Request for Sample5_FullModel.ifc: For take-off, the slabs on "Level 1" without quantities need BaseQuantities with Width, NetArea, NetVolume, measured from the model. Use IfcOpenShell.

First a look at what the model holds.

```python
import ifcopenshell
import ifcopenshell.util.element
import ifcopenshell.util.unit

model = ifcopenshell.open("Sample5_FullModel.ifc")
print(model.schema)
for unit_type in ("LENGTHUNIT", "AREAUNIT", "VOLUMEUNIT"):
    print(unit_type, ifcopenshell.util.unit.calculate_unit_scale(model, unit_type))
storey = next(s for s in model.by_type("IfcBuildingStorey") if s.Name == "Level 1")
slabs = [e for e in ifcopenshell.util.element.get_decomposition(storey) if e.is_a("IfcSlab")]
for e in sorted(slabs, key=lambda e: e.id()):
    print(e.id(), e.is_a(), e.Name, list(ifcopenshell.util.element.get_psets(e, qtos_only=True)), sep=" | ")
```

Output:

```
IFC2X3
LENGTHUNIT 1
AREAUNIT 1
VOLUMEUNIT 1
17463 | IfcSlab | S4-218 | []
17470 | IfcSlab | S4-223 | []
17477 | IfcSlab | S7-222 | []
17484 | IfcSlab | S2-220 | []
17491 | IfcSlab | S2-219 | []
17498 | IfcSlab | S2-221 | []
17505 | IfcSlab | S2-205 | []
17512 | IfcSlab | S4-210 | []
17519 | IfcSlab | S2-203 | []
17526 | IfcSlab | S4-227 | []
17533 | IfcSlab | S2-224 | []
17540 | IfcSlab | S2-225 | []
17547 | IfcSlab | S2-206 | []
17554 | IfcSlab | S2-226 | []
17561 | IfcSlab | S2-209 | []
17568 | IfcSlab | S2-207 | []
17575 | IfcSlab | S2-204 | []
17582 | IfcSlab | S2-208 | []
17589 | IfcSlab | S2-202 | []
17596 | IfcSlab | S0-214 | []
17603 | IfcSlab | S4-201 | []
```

```python
import ifcopenshell
import ifcopenshell.api.pset
import ifcopenshell.geom
import ifcopenshell.util.element
import ifcopenshell.util.shape
import ifcopenshell.util.unit

model = ifcopenshell.open("Sample5_FullModel.ifc")
unit_scale = ifcopenshell.util.unit.calculate_unit_scale(model)
area_scale = ifcopenshell.util.unit.calculate_unit_scale(model, "AREAUNIT")
volume_scale = ifcopenshell.util.unit.calculate_unit_scale(model, "VOLUMEUNIT")
settings = ifcopenshell.geom.settings()

storey = next(s for s in model.by_type("IfcBuildingStorey") if s.Name == "Level 1")
slabs = [e for e in ifcopenshell.util.element.get_decomposition(storey) if e.is_a("IfcSlab")]

for e in sorted(slabs, key=lambda e: e.id()):
    if ifcopenshell.util.element.get_psets(e, qtos_only=True, should_inherit=False):
        continue
    # Geometry comes back in metres, in the element's own axes.
    shape = ifcopenshell.geom.create_shape(settings, e)
    values = {
        "Width": ifcopenshell.util.shape.get_z(shape.geometry) / unit_scale,
        "NetArea": ifcopenshell.util.shape.get_footprint_area(shape.geometry) / area_scale,
        "NetVolume": ifcopenshell.util.shape.get_volume(shape.geometry) / volume_scale,
    }
    qto = ifcopenshell.api.pset.add_qto(model, product=e, name="BaseQuantities")
    ifcopenshell.api.pset.edit_qto(model, qto=qto, properties=values)
    print(e.id(), {k: round(v, 3) for k, v in values.items()})

model.write("Sample5_FullModel_edited.ifc")
```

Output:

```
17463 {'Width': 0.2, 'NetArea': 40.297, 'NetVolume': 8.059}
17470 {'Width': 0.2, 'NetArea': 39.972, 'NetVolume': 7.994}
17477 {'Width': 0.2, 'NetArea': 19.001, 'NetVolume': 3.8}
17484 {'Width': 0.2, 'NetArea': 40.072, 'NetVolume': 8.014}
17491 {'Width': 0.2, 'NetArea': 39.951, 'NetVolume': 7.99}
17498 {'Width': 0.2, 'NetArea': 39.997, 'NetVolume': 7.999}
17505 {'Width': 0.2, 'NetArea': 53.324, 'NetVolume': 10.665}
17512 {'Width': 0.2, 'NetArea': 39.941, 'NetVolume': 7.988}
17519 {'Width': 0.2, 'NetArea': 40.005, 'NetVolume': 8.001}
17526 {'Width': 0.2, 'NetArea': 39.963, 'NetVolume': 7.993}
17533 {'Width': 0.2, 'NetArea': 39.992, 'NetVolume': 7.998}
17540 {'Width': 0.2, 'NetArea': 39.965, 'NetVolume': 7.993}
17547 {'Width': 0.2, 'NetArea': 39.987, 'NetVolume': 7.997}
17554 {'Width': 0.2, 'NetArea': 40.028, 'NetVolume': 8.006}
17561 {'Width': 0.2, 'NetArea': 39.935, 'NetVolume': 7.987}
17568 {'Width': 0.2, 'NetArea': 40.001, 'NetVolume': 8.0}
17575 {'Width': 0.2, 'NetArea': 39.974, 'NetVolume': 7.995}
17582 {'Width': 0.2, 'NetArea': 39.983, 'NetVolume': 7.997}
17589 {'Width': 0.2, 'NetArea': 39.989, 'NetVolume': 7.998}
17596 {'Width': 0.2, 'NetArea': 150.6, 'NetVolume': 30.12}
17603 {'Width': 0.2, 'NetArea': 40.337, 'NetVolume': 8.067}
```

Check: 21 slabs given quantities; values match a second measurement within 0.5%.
